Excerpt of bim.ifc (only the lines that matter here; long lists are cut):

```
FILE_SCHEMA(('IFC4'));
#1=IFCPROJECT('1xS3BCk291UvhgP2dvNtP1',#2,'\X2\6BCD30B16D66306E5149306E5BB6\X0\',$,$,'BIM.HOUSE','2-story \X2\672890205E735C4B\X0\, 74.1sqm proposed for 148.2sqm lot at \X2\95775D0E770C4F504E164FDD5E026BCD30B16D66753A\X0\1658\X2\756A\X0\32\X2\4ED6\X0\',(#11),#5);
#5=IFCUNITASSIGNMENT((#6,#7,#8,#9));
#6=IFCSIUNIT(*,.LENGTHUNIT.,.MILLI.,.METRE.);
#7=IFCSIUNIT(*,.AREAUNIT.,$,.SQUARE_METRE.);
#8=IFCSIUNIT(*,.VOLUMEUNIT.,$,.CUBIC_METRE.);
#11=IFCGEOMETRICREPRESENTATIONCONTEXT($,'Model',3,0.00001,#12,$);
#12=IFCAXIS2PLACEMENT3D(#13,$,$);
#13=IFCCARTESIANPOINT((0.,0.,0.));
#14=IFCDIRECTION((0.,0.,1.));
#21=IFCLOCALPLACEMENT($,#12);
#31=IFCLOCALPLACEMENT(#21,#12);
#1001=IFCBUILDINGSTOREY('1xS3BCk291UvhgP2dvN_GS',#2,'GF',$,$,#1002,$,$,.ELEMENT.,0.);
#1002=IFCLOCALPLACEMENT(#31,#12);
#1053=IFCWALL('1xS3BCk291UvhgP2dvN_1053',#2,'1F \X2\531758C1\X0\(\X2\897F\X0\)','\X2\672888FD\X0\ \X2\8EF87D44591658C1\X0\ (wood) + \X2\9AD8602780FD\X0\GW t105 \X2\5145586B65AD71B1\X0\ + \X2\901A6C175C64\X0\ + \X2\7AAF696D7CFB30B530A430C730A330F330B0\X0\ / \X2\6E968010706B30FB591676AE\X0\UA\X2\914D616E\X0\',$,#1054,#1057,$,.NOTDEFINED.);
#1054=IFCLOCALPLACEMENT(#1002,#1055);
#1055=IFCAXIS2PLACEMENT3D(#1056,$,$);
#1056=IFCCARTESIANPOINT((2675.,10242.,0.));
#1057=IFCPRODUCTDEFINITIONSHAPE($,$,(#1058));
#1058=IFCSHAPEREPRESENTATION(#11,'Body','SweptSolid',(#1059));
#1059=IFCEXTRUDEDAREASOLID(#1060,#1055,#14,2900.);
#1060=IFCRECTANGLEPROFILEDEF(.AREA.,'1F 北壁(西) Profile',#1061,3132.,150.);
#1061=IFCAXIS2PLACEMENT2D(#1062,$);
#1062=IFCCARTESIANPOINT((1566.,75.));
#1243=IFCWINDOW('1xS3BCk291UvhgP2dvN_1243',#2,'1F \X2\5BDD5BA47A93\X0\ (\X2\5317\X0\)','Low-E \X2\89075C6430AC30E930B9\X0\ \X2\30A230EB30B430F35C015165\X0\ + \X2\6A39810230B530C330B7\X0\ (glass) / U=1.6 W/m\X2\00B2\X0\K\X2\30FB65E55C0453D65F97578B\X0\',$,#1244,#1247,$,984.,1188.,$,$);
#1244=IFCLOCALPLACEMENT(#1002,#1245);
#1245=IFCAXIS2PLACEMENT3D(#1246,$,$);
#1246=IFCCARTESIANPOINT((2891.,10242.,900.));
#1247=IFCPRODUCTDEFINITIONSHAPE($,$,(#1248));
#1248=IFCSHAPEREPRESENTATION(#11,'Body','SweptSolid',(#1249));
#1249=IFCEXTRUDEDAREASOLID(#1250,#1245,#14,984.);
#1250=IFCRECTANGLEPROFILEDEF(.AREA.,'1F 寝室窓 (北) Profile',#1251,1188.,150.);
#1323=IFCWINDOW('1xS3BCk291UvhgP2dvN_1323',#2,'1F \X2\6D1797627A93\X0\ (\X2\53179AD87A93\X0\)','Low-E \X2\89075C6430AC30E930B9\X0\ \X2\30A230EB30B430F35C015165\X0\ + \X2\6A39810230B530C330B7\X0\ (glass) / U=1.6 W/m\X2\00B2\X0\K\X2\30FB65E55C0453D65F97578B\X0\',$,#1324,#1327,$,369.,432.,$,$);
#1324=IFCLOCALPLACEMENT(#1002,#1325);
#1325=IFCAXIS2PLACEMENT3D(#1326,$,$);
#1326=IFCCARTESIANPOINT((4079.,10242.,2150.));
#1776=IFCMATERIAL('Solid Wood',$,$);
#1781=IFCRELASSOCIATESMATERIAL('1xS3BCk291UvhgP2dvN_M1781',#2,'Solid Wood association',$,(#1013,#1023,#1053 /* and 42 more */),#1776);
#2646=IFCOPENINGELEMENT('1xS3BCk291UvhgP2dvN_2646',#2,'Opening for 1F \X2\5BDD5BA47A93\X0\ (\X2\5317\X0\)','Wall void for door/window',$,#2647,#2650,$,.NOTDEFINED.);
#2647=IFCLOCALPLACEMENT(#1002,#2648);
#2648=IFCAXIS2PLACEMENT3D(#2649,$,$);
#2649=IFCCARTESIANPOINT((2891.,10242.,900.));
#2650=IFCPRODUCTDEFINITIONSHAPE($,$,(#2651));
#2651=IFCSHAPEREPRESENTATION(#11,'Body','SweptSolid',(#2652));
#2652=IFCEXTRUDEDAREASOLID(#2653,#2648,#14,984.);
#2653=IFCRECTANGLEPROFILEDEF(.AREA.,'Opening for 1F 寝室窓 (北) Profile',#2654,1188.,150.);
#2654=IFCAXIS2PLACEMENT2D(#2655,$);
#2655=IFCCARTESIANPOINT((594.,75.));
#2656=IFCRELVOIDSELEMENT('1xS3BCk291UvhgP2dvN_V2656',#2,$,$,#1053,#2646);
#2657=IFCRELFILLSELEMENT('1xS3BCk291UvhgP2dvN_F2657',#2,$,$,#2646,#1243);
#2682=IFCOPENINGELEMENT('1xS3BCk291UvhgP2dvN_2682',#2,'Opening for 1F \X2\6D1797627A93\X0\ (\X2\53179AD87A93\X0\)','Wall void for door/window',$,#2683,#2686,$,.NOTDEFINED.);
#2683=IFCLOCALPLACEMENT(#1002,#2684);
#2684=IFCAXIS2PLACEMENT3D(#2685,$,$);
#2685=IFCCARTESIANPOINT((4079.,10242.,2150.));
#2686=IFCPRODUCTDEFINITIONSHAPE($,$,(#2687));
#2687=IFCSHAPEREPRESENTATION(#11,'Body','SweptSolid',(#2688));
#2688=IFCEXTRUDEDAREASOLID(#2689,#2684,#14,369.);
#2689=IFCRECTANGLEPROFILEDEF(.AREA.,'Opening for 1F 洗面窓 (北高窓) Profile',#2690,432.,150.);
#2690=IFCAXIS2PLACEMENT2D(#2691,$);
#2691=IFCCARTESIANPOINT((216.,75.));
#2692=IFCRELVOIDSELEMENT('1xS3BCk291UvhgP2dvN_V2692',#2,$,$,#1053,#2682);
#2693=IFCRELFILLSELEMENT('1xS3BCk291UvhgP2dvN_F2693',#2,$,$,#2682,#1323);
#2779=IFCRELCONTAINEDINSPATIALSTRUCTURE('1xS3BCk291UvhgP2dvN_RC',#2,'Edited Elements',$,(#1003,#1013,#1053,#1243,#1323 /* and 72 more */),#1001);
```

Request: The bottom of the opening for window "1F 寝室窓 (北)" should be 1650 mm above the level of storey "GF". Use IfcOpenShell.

```python
import numpy as np
import ifcopenshell
import ifcopenshell.api.geometry
import ifcopenshell.geom
import ifcopenshell.util.element
import ifcopenshell.util.placement
import ifcopenshell.util.shape
import ifcopenshell.util.unit

model = ifcopenshell.open("bim.ifc")
unit_scale = ifcopenshell.util.unit.calculate_unit_scale(model)

window = model.by_id(1243)
opening = window.FillsVoids[0].RelatingOpeningElement
storey = ifcopenshell.util.element.get_container(window, ifc_class="IfcBuildingStorey")
level = ifcopenshell.util.placement.get_local_placement(storey.ObjectPlacement)[2, 3]

# The opening's origin need not be at the sill, so measure its lowest point.
shape = ifcopenshell.geom.create_shape(ifcopenshell.geom.settings(), opening)
bottom = ifcopenshell.util.shape.get_shape_bottom_elevation(shape, shape.geometry) / unit_scale
dz = level + 1650.0 - bottom

shift = np.array([0.0, 0.0, dz])
# The window is not placed relative to its opening, so move both.
for product in (opening, window):
    matrix = ifcopenshell.util.placement.get_local_placement(product.ObjectPlacement)
    matrix[:3, 3] += shift
    ifcopenshell.api.geometry.edit_object_placement(model, product=product, matrix=matrix, is_si=False)

print(f"moved by {dz * unit_scale:+.3f} m")

model.write("bim_edited.ifc")
```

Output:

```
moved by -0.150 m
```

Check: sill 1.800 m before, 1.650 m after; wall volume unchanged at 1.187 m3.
